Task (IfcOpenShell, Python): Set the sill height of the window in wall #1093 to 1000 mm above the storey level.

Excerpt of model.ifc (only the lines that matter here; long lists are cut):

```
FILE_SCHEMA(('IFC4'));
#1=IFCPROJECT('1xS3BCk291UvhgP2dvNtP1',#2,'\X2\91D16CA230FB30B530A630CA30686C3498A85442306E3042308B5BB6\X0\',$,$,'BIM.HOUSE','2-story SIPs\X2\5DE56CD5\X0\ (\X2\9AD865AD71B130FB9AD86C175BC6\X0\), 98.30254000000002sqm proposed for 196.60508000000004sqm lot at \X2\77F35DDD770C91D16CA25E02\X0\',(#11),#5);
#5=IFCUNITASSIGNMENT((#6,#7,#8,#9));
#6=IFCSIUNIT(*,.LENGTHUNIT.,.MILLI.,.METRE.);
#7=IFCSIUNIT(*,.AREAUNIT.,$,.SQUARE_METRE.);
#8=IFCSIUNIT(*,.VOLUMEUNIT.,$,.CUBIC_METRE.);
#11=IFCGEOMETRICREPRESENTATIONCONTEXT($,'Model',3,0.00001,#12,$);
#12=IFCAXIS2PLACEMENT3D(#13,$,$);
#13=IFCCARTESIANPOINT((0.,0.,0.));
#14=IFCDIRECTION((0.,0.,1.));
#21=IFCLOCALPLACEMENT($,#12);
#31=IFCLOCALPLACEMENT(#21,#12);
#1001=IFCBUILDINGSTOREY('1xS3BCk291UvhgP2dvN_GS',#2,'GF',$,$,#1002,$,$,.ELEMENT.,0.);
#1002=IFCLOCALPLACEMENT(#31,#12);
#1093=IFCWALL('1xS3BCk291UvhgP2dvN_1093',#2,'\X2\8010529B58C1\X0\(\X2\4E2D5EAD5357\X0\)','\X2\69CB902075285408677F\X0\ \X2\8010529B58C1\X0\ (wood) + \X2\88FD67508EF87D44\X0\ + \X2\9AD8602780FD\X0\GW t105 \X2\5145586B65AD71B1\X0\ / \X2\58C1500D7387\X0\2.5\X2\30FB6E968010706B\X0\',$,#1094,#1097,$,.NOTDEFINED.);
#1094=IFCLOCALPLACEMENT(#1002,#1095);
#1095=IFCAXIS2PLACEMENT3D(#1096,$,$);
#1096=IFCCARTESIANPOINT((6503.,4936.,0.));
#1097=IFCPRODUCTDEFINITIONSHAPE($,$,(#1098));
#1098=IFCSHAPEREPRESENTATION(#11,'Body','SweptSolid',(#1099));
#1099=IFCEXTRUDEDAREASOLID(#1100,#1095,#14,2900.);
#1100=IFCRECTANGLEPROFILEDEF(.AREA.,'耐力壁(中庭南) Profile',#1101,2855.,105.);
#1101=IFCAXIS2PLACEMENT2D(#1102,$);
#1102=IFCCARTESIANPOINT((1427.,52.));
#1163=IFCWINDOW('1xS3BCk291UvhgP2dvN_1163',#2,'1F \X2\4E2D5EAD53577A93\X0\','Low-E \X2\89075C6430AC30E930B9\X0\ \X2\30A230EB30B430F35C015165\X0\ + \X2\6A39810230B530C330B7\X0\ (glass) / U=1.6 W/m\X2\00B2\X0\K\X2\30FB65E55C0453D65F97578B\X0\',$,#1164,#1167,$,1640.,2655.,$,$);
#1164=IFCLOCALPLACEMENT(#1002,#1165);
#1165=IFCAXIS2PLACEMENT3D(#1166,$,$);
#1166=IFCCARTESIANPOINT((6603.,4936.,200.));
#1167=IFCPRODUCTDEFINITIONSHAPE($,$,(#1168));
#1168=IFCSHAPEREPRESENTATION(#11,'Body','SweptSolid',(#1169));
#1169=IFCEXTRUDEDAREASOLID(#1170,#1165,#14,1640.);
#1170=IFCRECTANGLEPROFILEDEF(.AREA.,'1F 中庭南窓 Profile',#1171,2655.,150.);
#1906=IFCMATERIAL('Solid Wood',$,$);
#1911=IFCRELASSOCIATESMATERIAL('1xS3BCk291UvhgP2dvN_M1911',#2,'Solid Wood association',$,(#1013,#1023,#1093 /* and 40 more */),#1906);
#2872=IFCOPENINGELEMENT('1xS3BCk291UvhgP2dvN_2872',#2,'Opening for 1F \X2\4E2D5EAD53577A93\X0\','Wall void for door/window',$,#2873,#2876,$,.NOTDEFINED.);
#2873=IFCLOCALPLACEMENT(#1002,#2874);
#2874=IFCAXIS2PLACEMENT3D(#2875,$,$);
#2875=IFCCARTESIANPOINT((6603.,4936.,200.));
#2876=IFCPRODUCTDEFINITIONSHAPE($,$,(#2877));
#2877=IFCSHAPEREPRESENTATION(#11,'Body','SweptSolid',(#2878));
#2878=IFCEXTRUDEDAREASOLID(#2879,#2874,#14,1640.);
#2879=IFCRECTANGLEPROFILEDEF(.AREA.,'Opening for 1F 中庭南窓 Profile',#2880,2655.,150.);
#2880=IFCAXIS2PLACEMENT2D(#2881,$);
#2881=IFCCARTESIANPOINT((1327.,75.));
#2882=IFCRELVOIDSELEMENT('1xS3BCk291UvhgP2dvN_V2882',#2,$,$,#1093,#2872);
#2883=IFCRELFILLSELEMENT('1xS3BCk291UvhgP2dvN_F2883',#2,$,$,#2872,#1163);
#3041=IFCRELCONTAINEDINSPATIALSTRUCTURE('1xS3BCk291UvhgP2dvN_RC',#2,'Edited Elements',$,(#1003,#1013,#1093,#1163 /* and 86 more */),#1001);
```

```python
import numpy as np
import ifcopenshell
import ifcopenshell.api.geometry
import ifcopenshell.geom
import ifcopenshell.util.element
import ifcopenshell.util.placement
import ifcopenshell.util.shape
import ifcopenshell.util.unit

model = ifcopenshell.open("model.ifc")
unit_scale = ifcopenshell.util.unit.calculate_unit_scale(model)

window = model.by_id(1163)
opening = window.FillsVoids[0].RelatingOpeningElement
storey = ifcopenshell.util.element.get_container(window, ifc_class="IfcBuildingStorey")
level = ifcopenshell.util.placement.get_local_placement(storey.ObjectPlacement)[2, 3]

# The opening's origin need not be at the sill, so measure its lowest point.
shape = ifcopenshell.geom.create_shape(ifcopenshell.geom.settings(), opening)
bottom = ifcopenshell.util.shape.get_shape_bottom_elevation(shape, shape.geometry) / unit_scale
dz = level + 1 / unit_scale - bottom

shift = np.array([0.0, 0.0, dz])
# The window is not placed relative to its opening, so move both.
for product in (opening, window):
    matrix = ifcopenshell.util.placement.get_local_placement(product.ObjectPlacement)
    matrix[:3, 3] += shift
    ifcopenshell.api.geometry.edit_object_placement(model, product=product, matrix=matrix, is_si=False)

print(f"moved by {dz * unit_scale:+.3f} m")

model.write("model_updated.ifc")
```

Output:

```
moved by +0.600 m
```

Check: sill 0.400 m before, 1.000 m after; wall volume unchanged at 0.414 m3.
